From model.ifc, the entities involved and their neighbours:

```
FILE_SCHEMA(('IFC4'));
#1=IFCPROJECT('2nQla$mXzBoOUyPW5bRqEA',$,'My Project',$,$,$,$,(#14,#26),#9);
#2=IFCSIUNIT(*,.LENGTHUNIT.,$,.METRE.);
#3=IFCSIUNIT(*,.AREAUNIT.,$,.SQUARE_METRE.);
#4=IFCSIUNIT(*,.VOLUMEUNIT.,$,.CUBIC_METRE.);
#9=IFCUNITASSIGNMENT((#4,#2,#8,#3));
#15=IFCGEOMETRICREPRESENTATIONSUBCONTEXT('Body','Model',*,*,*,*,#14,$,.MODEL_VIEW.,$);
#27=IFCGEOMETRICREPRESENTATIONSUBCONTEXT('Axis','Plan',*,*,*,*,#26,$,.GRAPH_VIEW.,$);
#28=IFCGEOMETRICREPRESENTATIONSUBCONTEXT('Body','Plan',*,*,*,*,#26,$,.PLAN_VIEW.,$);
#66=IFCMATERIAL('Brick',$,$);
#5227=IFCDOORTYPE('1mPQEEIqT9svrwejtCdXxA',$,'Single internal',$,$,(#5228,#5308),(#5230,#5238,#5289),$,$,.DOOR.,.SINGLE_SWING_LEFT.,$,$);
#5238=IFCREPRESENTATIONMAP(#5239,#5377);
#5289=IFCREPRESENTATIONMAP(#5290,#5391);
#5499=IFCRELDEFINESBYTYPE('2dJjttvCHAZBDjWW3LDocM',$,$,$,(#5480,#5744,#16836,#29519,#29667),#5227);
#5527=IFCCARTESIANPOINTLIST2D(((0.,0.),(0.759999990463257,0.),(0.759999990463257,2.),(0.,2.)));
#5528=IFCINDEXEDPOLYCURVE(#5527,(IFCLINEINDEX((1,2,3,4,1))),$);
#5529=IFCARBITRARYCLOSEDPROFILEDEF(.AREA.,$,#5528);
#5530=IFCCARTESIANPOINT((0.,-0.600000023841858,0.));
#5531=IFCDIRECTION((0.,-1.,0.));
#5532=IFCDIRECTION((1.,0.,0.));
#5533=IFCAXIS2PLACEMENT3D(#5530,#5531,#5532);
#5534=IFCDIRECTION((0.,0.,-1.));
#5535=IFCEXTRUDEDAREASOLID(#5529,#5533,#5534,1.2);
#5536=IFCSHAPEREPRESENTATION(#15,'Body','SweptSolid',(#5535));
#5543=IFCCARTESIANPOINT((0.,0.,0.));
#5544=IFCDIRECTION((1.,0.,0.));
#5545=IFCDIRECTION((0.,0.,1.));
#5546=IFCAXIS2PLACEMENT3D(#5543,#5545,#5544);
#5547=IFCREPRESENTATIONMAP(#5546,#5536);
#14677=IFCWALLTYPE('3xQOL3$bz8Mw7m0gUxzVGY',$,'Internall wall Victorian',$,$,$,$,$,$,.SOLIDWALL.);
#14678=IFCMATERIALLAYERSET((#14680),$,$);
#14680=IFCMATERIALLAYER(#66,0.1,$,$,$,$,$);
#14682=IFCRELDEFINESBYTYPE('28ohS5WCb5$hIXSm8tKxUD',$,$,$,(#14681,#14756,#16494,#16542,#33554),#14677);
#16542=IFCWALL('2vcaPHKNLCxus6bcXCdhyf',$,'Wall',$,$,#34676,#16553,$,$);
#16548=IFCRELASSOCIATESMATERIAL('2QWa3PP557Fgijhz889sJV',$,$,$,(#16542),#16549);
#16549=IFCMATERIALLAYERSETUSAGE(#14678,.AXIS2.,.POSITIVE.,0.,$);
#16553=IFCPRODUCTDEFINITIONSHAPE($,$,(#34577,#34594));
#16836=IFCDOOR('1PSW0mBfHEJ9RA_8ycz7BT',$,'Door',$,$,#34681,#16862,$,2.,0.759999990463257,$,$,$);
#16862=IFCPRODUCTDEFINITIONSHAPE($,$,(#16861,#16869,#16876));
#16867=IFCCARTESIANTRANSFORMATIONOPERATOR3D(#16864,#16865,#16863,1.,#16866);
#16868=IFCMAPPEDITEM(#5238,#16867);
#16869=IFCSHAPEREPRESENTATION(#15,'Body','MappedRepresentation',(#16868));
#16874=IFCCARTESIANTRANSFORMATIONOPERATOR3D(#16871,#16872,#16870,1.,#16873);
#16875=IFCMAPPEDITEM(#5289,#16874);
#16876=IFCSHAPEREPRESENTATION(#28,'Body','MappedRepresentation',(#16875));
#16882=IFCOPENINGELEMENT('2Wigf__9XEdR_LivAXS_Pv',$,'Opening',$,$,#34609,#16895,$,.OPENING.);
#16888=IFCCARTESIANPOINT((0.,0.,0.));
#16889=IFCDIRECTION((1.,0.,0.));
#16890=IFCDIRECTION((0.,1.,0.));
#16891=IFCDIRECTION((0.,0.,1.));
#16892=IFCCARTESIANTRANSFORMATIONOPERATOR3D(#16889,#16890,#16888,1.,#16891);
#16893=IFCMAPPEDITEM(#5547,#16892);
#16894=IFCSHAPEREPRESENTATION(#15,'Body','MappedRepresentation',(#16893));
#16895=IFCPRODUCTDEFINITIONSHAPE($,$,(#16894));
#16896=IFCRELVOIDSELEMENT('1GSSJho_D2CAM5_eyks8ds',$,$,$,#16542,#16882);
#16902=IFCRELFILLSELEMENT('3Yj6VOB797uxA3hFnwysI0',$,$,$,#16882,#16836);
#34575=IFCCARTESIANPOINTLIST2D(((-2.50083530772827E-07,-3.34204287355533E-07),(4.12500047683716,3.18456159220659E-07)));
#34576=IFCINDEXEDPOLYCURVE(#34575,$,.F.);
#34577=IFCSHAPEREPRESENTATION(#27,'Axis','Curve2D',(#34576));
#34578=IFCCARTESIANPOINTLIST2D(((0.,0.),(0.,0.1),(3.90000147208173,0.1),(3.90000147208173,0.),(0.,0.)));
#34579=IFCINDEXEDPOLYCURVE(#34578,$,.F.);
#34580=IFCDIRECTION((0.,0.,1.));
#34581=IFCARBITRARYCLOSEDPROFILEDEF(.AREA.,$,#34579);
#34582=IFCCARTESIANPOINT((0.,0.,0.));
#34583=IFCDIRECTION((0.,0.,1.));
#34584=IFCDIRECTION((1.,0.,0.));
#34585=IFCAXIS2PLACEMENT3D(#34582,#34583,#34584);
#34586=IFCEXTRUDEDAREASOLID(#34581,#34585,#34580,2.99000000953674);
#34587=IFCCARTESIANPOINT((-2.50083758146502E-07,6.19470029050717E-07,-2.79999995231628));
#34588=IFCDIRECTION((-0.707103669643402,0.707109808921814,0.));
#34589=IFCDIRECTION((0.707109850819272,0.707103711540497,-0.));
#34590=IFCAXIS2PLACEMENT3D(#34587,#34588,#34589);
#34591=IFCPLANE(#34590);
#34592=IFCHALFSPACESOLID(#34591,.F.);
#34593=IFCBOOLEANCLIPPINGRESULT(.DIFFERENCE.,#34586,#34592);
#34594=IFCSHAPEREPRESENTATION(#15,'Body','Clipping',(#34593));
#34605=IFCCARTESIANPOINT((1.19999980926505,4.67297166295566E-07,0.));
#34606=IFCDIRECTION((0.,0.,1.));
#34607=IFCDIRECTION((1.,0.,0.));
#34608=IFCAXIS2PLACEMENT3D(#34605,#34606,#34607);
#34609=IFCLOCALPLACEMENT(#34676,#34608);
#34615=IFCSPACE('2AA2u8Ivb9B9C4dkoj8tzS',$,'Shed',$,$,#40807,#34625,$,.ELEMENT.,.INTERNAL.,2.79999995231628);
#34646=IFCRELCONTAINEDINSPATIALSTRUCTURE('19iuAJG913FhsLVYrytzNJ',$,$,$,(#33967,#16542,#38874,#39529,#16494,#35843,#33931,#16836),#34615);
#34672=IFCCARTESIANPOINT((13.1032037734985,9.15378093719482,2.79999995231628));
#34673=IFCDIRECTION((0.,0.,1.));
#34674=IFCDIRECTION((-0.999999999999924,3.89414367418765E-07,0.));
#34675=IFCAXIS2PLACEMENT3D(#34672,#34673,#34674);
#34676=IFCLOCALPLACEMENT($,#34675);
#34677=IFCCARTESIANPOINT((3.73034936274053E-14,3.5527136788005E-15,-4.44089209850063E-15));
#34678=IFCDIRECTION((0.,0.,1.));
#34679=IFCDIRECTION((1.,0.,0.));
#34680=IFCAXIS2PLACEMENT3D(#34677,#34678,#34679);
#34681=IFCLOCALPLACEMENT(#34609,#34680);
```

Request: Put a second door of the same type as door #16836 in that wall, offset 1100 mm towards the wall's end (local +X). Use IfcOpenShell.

```python
import ifcopenshell
import ifcopenshell.api.feature
import ifcopenshell.api.geometry
import ifcopenshell.api.root
import ifcopenshell.geom
import ifcopenshell.util.element
import ifcopenshell.util.placement
import ifcopenshell.util.shape
import ifcopenshell.util.unit

model = ifcopenshell.open("model.ifc")
unit_scale = ifcopenshell.util.unit.calculate_unit_scale(model)
settings = ifcopenshell.geom.settings()


def volume(element):
    """Net volume in cubic metres, openings subtracted."""
    shape = ifcopenshell.geom.create_shape(settings, element)
    return ifcopenshell.util.shape.get_volume(shape.geometry)


door = model.by_guid("1PSW0mBfHEJ9RA_8ycz7BT")
opening = door.FillsVoids[0].RelatingOpeningElement
wall = opening.VoidsElements[0].RelatingBuildingElement
before = volume(wall)
shift = ifcopenshell.util.placement.get_local_placement(wall.ObjectPlacement)[:3, 0] * 1.1 / unit_scale

# copy_class copies the void relationship, type, container and properties, but no geometry.
new_opening = ifcopenshell.api.root.copy_class(model, product=opening)
new_opening.Representation = ifcopenshell.util.element.copy_deep(
    model, opening.Representation, exclude=["IfcGeometricRepresentationContext", "IfcRepresentationMap"]
)
new_door = ifcopenshell.api.root.copy_class(model, product=door)
new_door.Representation = ifcopenshell.util.element.copy_deep(
    model, door.Representation, exclude=["IfcGeometricRepresentationContext", "IfcRepresentationMap"]
)
ifcopenshell.api.feature.add_filling(model, opening=new_opening, element=new_door)

for old, new in ((opening, new_opening), (door, new_door)):
    matrix = ifcopenshell.util.placement.get_local_placement(old.ObjectPlacement)
    matrix[:3, 3] += shift
    ifcopenshell.api.geometry.edit_object_placement(model, product=new, matrix=matrix, is_si=False)

after = volume(wall)

print(f"wall volume {before:.3f} -> {after:.3f} m3")

model.write("model_v2.ifc")
```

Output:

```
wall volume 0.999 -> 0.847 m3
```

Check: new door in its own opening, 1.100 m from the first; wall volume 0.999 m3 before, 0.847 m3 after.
